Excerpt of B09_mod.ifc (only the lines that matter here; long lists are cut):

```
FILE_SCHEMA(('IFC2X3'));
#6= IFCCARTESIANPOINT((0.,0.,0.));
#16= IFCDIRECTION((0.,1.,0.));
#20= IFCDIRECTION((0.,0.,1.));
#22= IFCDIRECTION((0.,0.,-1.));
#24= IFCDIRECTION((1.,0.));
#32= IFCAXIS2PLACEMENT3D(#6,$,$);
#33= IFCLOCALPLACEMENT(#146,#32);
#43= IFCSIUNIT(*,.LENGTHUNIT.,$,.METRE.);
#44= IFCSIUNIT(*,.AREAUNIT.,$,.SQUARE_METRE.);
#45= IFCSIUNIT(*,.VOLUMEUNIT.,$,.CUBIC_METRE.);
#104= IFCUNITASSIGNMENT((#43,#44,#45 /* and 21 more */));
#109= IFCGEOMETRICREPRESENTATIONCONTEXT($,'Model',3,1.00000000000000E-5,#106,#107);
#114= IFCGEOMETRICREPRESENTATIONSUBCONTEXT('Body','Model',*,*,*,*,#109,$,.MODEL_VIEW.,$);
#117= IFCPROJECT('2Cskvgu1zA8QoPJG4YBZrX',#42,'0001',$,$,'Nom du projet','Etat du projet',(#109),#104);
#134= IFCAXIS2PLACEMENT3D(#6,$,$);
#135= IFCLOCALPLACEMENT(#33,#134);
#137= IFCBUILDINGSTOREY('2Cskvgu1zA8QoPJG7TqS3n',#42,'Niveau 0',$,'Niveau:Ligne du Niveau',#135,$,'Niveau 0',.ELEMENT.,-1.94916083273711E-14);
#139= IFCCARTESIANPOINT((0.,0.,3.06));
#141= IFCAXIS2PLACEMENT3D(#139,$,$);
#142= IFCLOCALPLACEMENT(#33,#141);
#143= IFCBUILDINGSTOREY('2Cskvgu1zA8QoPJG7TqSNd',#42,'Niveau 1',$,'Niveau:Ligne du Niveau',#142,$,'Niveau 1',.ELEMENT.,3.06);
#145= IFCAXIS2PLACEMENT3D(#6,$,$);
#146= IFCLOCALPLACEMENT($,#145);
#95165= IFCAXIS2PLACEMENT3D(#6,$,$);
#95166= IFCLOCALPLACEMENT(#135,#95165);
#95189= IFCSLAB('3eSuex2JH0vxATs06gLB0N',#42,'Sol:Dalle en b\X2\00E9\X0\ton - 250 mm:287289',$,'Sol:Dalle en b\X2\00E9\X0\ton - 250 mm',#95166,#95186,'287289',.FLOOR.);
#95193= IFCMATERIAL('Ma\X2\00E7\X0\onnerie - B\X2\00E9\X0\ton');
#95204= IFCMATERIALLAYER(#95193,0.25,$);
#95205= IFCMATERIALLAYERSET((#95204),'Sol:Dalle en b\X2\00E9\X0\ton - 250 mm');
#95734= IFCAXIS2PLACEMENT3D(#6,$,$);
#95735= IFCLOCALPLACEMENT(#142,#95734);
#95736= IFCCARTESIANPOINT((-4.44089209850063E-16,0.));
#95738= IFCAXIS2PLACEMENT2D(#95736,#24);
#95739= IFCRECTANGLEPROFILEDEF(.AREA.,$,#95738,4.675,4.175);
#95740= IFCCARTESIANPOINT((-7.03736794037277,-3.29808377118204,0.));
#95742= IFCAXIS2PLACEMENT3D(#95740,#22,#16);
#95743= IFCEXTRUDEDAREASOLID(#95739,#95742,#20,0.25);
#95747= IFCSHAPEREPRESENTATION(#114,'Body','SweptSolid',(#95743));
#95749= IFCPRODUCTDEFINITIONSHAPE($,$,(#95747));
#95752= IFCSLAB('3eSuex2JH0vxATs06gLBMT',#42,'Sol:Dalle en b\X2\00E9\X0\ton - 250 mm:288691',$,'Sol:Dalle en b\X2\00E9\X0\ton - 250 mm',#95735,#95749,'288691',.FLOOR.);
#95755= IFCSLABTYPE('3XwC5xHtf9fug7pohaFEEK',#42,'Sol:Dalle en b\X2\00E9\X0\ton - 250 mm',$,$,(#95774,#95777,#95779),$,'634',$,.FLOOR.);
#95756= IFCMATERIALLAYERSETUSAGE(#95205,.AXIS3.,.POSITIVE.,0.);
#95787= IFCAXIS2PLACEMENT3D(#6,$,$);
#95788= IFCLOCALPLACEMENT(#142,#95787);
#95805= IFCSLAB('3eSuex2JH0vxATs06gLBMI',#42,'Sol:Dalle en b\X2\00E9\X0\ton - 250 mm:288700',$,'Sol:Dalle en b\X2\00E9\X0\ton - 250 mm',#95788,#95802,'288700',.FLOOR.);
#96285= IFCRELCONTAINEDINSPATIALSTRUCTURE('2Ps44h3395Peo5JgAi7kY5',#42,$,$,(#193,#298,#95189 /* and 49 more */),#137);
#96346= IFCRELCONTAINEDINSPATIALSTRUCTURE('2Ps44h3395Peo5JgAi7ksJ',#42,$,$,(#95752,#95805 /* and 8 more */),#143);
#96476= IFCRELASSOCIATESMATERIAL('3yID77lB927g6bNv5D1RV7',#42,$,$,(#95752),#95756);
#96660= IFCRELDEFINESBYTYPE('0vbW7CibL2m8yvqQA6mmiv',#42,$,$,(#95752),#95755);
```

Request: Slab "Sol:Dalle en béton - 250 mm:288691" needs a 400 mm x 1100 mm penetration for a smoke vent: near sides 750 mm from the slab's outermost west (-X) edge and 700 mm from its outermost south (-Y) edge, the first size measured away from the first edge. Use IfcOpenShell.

```python
import numpy as np
import ifcopenshell
import ifcopenshell.api.feature
import ifcopenshell.api.geometry
import ifcopenshell.api.root
import ifcopenshell.geom
import ifcopenshell.util.placement
import ifcopenshell.util.representation
import ifcopenshell.util.shape
import ifcopenshell.util.unit

model = ifcopenshell.open("B09_mod.ifc")
unit_scale = ifcopenshell.util.unit.calculate_unit_scale(model)
settings = ifcopenshell.geom.settings()


def volume(element):
    """Net volume in cubic metres, openings subtracted."""
    shape = ifcopenshell.geom.create_shape(settings, element)
    return ifcopenshell.util.shape.get_volume(shape.geometry)


slab = model.by_id(95752)
before = volume(slab)

# Extent in the slab's own axes, in metres. The edges named are its -X and -Y sides.
slab_shape = ifcopenshell.geom.create_shape(settings, slab)
vertices = ifcopenshell.util.shape.get_vertices(slab_shape.geometry)
x_min, y_min, bottom = vertices.min(axis=0)
top = vertices[:, 2].max()

opening = ifcopenshell.api.root.create_entity(model, ifc_class="IfcOpeningElement", name="Smoke vent opening")
context = ifcopenshell.util.representation.get_context(model, "Model", "Body", "MODEL_VIEW")
width, depth = 0.4, 1.1
outline = [(0.0, 0.0), (width, 0.0), (width, depth), (0.0, depth), (0.0, 0.0)]
# Overshoot both faces by 50 mm so the cut is clean.
shape = ifcopenshell.api.geometry.add_slab_representation(
    model, context=context, depth=top - bottom + 0.1, polyline=outline
)
ifcopenshell.api.geometry.assign_representation(model, product=opening, representation=shape)

matrix = ifcopenshell.util.placement.get_local_placement(slab.ObjectPlacement)
matrix[:, 3] = matrix @ np.append(np.array([x_min + 0.75, y_min + 0.7, bottom - 0.05]) / unit_scale, 1.0)
ifcopenshell.api.geometry.edit_object_placement(model, product=opening, matrix=matrix, is_si=False)
ifcopenshell.api.feature.add_feature(model, feature=opening, element=slab)

after = volume(slab)

print(f"slab volume {before:.3f} -> {after:.3f} m3")

model.write("B09_mod-out.ifc")
```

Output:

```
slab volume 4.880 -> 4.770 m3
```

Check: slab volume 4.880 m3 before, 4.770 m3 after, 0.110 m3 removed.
